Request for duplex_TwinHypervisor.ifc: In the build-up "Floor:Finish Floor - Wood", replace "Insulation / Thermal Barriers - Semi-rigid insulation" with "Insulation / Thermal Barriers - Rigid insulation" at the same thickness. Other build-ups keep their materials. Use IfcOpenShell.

First a look at what the model holds.

```python
import ifcopenshell
import ifcopenshell.util.element

model = ifcopenshell.open("duplex_TwinHypervisor.ifc")
print(model.schema)
for layer_set in model.by_type("IfcMaterialLayerSet"):
    if layer_set.LayerSetName == "Floor:Finish Floor - Wood":
        for layer in layer_set.MaterialLayers:
            print(layer.id(), layer.Material and layer.Material.Name, layer.LayerThickness, sep=" | ")
        print(len(ifcopenshell.util.element.get_elements_by_material(model, layer_set)), "elements and types use it")
print(sorted(m.Name for m in model.by_type("IfcMaterial") if m.Name)[:60])
```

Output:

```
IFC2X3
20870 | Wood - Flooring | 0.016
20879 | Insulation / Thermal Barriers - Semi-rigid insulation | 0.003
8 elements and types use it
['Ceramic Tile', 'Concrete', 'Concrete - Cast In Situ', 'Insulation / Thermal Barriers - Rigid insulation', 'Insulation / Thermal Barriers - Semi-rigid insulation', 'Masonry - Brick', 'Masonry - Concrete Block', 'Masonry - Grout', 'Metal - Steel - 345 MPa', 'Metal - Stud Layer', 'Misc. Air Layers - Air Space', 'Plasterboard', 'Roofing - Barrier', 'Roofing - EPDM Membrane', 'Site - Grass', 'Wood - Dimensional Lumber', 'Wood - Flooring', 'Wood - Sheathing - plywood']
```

```python
import ifcopenshell
import ifcopenshell.api.material

model = ifcopenshell.open("duplex_TwinHypervisor.ifc")

layer_set = next(s for s in model.by_type("IfcMaterialLayerSet") if s.LayerSetName == "Floor:Finish Floor - Wood")
layer = next(l for l in layer_set.MaterialLayers if l.Material and l.Material.Name == "Insulation / Thermal Barriers - Semi-rigid insulation")
material = next(m for m in model.by_type("IfcMaterial") if m.Name == "Insulation / Thermal Barriers - Rigid insulation")

# Point this one layer at the other material; renaming the old one would change it everywhere.
ifcopenshell.api.material.edit_layer(model, layer=layer, attributes={}, material=material)

print([l.Material.Name if l.Material else None for l in layer_set.MaterialLayers])

model.write("duplex_TwinHypervisor_rev.ifc")
```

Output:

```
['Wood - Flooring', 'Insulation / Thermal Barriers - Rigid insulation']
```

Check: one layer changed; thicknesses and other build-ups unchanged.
